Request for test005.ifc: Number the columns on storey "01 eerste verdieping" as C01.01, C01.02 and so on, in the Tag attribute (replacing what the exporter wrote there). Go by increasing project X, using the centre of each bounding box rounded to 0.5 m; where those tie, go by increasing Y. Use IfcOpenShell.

First a look at what the model holds.

```python
import ifcopenshell
import ifcopenshell.util.element
import ifcopenshell.util.placement

model = ifcopenshell.open("test005.ifc")
print(model.schema)
storey = next(s for s in model.by_type("IfcBuildingStorey") if s.Name == "01 eerste verdieping")
columns = [e for e in ifcopenshell.util.element.get_decomposition(storey) if e.is_a("IfcColumn")]
for e in sorted(columns, key=lambda e: e.id()):
    origin = ifcopenshell.util.placement.get_local_placement(e.ObjectPlacement)[:3, 3]
    print(e.id(), e.Tag, e.Name, origin.round(2) + 0.0, sep=" | ")
```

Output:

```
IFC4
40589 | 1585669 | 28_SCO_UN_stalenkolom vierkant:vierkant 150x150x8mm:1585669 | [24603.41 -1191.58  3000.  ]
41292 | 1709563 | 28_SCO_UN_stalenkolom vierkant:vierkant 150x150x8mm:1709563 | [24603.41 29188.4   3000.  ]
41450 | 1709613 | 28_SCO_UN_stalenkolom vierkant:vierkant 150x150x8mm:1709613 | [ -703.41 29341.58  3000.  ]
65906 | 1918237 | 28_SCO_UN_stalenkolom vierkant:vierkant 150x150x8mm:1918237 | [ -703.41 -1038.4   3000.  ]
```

```python
import ifcopenshell
import ifcopenshell.geom
import ifcopenshell.util.element
import ifcopenshell.util.shape

model = ifcopenshell.open("test005.ifc")
settings = ifcopenshell.geom.settings()
settings.set("use-world-coords", True)


def centre(element):
    shape = ifcopenshell.geom.create_shape(settings, element)
    return ifcopenshell.util.shape.get_bbox_centroid(shape.geometry)


storey = next(s for s in model.by_type("IfcBuildingStorey") if s.Name == "01 eerste verdieping")
columns = [e for e in ifcopenshell.util.element.get_decomposition(storey) if e.is_a("IfcColumn")]

# Insertion points can sit at a corner or the storey origin, so sort by the geometry (in metres).
centres = {e: centre(e) for e in columns}
columns.sort(key=lambda e: (round(centres[e][0] / 0.5), centres[e][1]))

for i, e in enumerate(columns, start=1):
    number = f"C01.{i:02d}"
    e.Tag = number
    print(e.id(), number)

model.write("test005_updated.ifc")
```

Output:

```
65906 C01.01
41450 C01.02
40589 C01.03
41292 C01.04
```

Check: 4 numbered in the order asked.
